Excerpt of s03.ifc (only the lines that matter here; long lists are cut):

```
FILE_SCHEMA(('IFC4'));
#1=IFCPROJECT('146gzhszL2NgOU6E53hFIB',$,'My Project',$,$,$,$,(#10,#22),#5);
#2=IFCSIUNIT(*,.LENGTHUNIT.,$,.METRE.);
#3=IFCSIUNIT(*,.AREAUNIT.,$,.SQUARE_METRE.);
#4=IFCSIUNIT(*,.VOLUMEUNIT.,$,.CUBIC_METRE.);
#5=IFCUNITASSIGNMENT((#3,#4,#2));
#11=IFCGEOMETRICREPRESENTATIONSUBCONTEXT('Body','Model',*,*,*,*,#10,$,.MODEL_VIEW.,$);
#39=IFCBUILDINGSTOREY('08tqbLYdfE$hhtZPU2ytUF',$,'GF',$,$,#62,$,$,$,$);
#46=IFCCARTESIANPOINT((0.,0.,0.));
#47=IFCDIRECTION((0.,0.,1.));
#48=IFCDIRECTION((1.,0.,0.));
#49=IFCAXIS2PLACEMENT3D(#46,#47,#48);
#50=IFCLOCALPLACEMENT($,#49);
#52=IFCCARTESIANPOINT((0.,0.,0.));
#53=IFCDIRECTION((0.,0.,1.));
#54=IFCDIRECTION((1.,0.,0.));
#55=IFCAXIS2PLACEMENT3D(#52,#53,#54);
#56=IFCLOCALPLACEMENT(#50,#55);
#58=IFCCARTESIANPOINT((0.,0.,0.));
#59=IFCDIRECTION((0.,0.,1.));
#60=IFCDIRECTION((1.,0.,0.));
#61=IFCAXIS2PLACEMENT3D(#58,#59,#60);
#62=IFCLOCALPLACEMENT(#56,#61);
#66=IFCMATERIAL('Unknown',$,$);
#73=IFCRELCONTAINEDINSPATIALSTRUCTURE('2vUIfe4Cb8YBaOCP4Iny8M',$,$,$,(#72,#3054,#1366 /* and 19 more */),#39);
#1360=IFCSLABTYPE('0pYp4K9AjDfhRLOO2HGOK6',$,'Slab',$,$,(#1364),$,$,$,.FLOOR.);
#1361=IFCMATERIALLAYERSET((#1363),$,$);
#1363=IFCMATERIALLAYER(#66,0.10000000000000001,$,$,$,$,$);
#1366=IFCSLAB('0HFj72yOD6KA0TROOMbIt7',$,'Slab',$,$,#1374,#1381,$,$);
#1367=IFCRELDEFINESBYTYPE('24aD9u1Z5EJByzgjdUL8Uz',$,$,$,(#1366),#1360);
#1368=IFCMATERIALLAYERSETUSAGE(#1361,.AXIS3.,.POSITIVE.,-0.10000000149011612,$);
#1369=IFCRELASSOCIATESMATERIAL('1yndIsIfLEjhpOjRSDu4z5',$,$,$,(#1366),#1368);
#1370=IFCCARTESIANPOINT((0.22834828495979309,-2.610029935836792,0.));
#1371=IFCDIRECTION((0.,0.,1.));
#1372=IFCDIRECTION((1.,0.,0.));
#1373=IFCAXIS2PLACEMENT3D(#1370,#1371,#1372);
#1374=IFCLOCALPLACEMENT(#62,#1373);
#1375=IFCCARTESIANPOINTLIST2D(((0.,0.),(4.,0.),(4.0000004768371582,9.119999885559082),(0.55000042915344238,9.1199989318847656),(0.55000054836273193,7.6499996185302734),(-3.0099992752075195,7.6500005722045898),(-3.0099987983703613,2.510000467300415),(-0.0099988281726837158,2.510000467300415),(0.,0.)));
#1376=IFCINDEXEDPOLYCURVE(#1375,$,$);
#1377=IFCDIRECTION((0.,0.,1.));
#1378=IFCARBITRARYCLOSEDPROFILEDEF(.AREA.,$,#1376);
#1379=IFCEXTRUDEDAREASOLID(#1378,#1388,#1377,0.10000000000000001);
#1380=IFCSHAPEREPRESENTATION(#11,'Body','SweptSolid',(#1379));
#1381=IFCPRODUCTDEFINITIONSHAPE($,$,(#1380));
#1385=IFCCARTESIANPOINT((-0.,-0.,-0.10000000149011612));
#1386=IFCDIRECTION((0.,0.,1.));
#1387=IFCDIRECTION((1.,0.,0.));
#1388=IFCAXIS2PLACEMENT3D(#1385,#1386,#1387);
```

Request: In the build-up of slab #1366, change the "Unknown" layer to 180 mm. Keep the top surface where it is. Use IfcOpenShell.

```python
import ifcopenshell
import ifcopenshell.util.element
import ifcopenshell.util.representation
import ifcopenshell.util.unit

model = ifcopenshell.open("s03.ifc")
unit_scale = ifcopenshell.util.unit.calculate_unit_scale(model)

layer_set = model.by_id(1361)
layer = next(l for l in layer_set.MaterialLayers if l.Material and l.Material.Name == "Unknown")
change = 0.18 / unit_scale - layer.LayerThickness
layer.LayerThickness += change

# Geometry does not follow the layer set by itself.
slabs = [e for e in ifcopenshell.util.element.get_elements_by_material(model, layer_set) if e.is_a("IfcSlab")]
for slab in sorted(slabs, key=lambda e: e.id()):
    body = ifcopenshell.util.representation.get_representation(slab, "Model", "Body")
    solid = body.Items[0]
    old_depth = solid.Depth
    solid.Depth += change
    # Extruded upwards: lower the start of the extrusion so the top stays.
    x, y, z = solid.Position.Location.Coordinates
    solid.Position.Location = model.createIfcCartesianPoint((x, y, z - change))
    print(slab.id(), f"{old_depth:g} -> {solid.Depth:g}")

# The layers are counted up from the underside, which has moved.
for usage in {ifcopenshell.util.element.get_material(slab) for slab in slabs}:
    usage.OffsetFromReferenceLine -= change

model.write("s03_v2.ifc")
```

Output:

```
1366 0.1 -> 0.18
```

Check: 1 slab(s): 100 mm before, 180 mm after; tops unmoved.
